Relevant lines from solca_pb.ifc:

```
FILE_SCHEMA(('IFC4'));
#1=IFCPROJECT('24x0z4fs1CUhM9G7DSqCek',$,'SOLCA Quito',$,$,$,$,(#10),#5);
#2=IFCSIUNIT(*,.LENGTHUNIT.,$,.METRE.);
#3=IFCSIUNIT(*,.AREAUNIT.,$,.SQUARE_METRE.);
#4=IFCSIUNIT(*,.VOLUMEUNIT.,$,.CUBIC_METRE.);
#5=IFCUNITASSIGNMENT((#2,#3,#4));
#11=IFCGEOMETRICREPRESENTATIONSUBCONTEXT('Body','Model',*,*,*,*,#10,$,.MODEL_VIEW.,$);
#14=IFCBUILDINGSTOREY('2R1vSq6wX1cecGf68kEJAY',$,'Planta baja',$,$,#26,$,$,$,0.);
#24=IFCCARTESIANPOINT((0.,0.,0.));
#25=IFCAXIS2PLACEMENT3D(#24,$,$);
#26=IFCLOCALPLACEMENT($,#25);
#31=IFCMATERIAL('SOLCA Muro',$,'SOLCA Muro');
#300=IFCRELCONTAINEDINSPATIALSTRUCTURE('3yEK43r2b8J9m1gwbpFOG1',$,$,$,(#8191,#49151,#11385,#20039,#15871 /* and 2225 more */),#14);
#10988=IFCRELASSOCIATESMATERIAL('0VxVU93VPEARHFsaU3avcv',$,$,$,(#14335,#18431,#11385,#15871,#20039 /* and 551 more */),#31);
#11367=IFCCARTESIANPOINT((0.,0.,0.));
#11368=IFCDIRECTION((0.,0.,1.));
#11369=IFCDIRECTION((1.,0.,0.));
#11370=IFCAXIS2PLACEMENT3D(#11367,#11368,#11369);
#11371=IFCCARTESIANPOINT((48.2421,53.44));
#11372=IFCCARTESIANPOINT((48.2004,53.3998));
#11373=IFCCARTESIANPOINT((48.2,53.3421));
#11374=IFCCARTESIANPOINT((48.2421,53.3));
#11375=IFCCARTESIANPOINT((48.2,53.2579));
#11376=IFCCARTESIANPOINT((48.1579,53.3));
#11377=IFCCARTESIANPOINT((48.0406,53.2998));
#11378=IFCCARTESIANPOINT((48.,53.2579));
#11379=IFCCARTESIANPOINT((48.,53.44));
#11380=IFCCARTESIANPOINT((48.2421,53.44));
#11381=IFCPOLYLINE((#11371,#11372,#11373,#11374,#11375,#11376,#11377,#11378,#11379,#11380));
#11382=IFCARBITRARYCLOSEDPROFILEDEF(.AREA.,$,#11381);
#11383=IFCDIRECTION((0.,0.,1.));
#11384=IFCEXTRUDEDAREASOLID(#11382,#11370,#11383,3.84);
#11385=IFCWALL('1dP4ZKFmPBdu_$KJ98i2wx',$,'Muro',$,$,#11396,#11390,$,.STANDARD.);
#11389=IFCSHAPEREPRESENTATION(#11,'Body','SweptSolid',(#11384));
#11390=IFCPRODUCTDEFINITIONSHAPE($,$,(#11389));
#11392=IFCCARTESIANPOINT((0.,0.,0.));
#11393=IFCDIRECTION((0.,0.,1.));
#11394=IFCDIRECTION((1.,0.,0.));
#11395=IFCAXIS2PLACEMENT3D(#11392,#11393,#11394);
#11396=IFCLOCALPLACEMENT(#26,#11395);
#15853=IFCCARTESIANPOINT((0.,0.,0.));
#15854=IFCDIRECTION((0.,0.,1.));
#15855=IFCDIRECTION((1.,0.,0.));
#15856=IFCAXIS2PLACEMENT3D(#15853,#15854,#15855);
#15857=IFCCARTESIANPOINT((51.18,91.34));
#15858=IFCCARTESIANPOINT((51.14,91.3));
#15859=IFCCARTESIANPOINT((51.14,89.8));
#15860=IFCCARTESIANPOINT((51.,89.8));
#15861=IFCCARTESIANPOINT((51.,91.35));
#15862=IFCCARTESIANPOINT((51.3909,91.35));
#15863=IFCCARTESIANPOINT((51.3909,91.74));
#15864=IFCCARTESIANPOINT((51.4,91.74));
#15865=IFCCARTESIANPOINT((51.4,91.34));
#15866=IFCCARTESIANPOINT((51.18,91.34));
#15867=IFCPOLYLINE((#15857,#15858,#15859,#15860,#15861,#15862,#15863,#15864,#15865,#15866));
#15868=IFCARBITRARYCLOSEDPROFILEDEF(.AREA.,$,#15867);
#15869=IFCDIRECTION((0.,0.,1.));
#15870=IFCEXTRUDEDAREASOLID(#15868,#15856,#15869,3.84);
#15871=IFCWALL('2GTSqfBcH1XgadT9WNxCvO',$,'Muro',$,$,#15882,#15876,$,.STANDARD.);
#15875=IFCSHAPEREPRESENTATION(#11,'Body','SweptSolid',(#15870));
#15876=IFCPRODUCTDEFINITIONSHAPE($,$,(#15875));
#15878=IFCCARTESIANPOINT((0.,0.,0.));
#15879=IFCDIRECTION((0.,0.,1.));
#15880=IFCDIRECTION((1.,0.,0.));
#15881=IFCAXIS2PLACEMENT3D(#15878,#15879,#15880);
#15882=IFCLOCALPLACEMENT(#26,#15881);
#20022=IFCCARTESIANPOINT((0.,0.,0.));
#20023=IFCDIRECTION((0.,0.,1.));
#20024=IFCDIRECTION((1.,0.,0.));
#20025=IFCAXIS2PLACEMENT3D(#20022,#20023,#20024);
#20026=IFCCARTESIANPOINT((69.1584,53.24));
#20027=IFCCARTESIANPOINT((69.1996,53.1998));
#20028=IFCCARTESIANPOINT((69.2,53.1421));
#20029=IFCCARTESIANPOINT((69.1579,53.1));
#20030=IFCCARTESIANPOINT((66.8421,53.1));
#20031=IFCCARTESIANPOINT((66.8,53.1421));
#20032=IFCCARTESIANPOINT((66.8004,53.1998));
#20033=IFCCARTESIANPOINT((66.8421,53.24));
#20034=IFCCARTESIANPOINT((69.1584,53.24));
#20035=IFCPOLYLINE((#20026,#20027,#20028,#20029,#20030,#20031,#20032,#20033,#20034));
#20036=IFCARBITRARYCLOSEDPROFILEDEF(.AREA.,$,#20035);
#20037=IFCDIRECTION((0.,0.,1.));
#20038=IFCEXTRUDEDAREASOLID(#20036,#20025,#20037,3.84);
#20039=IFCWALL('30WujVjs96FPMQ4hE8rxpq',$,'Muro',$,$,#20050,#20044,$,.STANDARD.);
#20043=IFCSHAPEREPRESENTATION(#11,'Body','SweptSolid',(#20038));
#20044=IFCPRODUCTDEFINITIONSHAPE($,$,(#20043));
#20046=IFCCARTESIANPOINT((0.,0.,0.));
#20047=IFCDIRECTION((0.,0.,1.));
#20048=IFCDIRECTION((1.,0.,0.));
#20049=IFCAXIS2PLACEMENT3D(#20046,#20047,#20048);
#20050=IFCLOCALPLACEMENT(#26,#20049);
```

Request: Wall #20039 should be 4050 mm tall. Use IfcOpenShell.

```python
import ifcopenshell
import ifcopenshell.geom
import ifcopenshell.util.representation
import ifcopenshell.util.shape

model = ifcopenshell.open("solca_pb.ifc")
settings = ifcopenshell.geom.settings()


def volume(element):
    """Net volume in cubic metres, openings subtracted."""
    shape = ifcopenshell.geom.create_shape(settings, element)
    return ifcopenshell.util.shape.get_volume(shape.geometry)


wall = model.by_id(20039)
before = volume(wall)

body = ifcopenshell.util.representation.get_representation(wall, "Model", "Body")
solid = body.Items[0]
old_height = solid.Depth
solid.Depth = 4.05
after = volume(wall)

print(f"height {old_height:g} -> {solid.Depth:g}, volume {before:.3f} -> {after:.3f} m3")

model.write("solca_pb_v2.ifc")
```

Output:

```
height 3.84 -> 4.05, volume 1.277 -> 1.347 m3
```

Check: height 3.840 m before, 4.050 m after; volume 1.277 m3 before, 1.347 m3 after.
